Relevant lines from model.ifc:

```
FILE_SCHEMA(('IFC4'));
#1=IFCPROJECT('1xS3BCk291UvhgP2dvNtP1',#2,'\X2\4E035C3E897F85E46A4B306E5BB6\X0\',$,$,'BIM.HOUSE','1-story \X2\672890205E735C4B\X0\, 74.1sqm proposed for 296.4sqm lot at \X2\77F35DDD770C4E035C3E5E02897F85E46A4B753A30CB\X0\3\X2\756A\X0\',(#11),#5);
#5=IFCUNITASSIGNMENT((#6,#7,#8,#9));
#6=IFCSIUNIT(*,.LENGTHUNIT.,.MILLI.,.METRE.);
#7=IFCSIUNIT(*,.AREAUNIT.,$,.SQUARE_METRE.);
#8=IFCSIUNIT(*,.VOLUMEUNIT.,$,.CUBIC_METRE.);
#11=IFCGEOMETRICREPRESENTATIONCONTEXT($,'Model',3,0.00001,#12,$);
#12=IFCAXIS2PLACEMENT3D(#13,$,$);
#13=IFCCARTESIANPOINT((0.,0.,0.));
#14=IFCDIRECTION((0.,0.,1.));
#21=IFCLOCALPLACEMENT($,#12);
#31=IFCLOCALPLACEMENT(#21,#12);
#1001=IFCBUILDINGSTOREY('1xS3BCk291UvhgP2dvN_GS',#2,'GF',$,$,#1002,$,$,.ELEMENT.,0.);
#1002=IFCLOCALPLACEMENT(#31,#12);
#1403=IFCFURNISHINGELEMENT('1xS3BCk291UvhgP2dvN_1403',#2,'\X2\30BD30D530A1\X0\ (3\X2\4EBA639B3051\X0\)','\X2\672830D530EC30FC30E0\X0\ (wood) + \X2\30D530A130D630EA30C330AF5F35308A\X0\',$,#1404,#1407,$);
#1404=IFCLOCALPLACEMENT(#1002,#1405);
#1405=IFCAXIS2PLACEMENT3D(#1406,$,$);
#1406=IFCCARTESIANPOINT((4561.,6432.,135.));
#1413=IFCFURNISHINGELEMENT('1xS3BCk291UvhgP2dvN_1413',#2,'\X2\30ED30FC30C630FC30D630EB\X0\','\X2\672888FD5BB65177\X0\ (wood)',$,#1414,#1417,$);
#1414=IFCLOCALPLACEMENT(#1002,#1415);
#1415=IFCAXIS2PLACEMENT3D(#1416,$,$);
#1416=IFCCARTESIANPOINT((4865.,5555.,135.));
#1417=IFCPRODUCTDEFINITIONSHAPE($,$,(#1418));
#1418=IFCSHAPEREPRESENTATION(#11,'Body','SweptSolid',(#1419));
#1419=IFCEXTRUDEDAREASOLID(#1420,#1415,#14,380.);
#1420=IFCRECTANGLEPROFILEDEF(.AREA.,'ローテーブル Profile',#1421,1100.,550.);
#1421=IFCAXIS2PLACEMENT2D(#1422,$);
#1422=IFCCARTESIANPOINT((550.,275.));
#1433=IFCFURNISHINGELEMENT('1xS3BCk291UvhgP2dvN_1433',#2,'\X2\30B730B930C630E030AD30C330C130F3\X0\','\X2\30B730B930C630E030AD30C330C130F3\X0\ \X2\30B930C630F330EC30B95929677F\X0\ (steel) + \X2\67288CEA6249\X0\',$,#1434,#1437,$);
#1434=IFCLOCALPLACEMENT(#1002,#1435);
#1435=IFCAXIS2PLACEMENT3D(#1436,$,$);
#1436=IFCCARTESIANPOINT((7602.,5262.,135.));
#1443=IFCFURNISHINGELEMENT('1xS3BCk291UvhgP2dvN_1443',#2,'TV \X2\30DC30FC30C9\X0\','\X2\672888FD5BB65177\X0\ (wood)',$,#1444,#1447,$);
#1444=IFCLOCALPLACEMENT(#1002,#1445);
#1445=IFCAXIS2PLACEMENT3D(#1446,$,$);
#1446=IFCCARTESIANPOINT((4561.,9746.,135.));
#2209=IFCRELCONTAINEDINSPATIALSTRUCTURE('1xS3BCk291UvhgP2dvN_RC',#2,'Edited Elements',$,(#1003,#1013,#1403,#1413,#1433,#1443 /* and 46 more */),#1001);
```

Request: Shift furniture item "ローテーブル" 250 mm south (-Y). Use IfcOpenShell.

```python
import ifcopenshell
import ifcopenshell.api.geometry
import ifcopenshell.util.placement

model = ifcopenshell.open("model.ifc")

item = model.by_id(1413)
matrix = ifcopenshell.util.placement.get_local_placement(item.ObjectPlacement)
matrix[1, 3] -= 250.0
ifcopenshell.api.geometry.edit_object_placement(model, product=item, matrix=matrix, is_si=False)

print(ifcopenshell.util.placement.get_local_placement(item.ObjectPlacement).round(3) + 0.0)

model.write("model_edited.ifc")
```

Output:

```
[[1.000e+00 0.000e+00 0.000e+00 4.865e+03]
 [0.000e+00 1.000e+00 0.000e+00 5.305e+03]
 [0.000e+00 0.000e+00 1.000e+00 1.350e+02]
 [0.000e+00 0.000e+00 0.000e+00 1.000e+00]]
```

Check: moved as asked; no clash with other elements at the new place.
